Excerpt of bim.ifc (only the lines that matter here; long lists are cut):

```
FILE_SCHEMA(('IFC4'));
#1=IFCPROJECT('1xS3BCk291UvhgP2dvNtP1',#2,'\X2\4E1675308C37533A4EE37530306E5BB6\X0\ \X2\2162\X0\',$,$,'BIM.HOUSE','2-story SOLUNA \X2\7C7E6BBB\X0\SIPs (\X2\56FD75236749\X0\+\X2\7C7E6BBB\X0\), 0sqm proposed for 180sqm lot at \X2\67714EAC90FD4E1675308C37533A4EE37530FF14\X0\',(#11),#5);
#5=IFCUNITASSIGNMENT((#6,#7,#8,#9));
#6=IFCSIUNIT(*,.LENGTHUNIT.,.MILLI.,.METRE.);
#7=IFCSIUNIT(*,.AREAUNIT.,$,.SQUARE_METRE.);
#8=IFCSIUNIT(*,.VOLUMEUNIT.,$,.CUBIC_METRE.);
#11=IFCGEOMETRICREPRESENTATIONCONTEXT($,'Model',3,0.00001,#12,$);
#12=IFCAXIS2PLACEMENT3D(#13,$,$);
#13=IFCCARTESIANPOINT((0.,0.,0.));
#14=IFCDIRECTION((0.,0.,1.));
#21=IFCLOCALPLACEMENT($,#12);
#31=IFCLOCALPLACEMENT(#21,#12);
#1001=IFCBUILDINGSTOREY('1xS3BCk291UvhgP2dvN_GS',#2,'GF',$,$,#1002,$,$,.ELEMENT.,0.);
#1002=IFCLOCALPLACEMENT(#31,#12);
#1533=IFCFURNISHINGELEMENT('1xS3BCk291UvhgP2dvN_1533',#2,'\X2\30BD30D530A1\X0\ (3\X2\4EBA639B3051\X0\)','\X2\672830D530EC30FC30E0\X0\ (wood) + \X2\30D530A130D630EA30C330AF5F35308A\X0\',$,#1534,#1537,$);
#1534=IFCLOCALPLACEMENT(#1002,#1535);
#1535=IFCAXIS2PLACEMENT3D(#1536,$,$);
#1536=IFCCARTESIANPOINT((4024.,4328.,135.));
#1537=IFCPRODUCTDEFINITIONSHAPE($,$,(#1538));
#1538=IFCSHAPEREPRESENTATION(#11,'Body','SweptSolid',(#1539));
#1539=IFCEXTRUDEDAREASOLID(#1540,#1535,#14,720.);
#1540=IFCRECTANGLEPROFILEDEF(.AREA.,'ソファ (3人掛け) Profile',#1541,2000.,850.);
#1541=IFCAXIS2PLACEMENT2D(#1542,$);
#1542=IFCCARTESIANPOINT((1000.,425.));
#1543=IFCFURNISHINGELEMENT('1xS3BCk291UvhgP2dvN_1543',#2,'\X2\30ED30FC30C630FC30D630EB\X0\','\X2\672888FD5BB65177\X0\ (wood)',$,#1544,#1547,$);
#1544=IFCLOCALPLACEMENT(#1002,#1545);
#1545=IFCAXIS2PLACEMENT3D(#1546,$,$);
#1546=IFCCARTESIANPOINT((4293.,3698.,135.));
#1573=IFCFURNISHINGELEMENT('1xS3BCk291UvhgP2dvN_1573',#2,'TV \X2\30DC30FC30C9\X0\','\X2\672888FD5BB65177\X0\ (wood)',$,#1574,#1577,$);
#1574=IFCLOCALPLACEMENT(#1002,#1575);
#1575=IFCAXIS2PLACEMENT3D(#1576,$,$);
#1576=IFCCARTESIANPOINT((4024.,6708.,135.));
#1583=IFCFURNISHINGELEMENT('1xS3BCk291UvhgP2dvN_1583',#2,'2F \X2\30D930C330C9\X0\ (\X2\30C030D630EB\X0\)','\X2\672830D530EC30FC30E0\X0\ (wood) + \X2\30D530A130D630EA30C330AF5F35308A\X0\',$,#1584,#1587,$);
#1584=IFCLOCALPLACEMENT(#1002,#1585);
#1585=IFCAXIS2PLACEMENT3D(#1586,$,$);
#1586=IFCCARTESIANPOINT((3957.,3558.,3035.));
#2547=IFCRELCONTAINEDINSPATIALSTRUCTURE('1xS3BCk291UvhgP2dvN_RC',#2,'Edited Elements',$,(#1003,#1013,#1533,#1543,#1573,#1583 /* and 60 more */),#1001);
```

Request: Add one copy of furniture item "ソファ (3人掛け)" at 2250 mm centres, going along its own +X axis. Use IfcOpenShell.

```python
import ifcopenshell
import ifcopenshell.api.geometry
import ifcopenshell.api.root
import ifcopenshell.util.element
import ifcopenshell.util.placement
import ifcopenshell.util.unit

model = ifcopenshell.open("bim.ifc")
unit_scale = ifcopenshell.util.unit.calculate_unit_scale(model)


def reuse_history(source, copy):
    """copy_class also copies each property set's owner history, people and application; keep the originals."""
    for rel in copy.IsDefinedBy:
        if rel.is_a("IfcRelDefinesByProperties") and (history := rel.RelatingPropertyDefinition.OwnerHistory):
            rel.RelatingPropertyDefinition.OwnerHistory = source.OwnerHistory
            ifcopenshell.util.element.remove_deep2(model, history)


source = model.by_guid("1xS3BCk291UvhgP2dvN_1533")
base = ifcopenshell.util.placement.get_local_placement(source.ObjectPlacement)
step = base[:3, 0] * 2.25 / unit_scale

for i in range(1, 2):
    copy = ifcopenshell.api.root.copy_class(model, product=source)
    copy.Representation = ifcopenshell.util.element.copy_deep(
        model, source.Representation, exclude=["IfcGeometricRepresentationContext", "IfcRepresentationMap"]
    )
    reuse_history(source, copy)
    matrix = base.copy()
    matrix[:3, 3] += i * step
    print("added at", matrix[:3, 3].round(3) + 0.0)
    ifcopenshell.api.geometry.edit_object_placement(model, product=copy, matrix=matrix, is_si=False)

model.write("bim_rev.ifc")
```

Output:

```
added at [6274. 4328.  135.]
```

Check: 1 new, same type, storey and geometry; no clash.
